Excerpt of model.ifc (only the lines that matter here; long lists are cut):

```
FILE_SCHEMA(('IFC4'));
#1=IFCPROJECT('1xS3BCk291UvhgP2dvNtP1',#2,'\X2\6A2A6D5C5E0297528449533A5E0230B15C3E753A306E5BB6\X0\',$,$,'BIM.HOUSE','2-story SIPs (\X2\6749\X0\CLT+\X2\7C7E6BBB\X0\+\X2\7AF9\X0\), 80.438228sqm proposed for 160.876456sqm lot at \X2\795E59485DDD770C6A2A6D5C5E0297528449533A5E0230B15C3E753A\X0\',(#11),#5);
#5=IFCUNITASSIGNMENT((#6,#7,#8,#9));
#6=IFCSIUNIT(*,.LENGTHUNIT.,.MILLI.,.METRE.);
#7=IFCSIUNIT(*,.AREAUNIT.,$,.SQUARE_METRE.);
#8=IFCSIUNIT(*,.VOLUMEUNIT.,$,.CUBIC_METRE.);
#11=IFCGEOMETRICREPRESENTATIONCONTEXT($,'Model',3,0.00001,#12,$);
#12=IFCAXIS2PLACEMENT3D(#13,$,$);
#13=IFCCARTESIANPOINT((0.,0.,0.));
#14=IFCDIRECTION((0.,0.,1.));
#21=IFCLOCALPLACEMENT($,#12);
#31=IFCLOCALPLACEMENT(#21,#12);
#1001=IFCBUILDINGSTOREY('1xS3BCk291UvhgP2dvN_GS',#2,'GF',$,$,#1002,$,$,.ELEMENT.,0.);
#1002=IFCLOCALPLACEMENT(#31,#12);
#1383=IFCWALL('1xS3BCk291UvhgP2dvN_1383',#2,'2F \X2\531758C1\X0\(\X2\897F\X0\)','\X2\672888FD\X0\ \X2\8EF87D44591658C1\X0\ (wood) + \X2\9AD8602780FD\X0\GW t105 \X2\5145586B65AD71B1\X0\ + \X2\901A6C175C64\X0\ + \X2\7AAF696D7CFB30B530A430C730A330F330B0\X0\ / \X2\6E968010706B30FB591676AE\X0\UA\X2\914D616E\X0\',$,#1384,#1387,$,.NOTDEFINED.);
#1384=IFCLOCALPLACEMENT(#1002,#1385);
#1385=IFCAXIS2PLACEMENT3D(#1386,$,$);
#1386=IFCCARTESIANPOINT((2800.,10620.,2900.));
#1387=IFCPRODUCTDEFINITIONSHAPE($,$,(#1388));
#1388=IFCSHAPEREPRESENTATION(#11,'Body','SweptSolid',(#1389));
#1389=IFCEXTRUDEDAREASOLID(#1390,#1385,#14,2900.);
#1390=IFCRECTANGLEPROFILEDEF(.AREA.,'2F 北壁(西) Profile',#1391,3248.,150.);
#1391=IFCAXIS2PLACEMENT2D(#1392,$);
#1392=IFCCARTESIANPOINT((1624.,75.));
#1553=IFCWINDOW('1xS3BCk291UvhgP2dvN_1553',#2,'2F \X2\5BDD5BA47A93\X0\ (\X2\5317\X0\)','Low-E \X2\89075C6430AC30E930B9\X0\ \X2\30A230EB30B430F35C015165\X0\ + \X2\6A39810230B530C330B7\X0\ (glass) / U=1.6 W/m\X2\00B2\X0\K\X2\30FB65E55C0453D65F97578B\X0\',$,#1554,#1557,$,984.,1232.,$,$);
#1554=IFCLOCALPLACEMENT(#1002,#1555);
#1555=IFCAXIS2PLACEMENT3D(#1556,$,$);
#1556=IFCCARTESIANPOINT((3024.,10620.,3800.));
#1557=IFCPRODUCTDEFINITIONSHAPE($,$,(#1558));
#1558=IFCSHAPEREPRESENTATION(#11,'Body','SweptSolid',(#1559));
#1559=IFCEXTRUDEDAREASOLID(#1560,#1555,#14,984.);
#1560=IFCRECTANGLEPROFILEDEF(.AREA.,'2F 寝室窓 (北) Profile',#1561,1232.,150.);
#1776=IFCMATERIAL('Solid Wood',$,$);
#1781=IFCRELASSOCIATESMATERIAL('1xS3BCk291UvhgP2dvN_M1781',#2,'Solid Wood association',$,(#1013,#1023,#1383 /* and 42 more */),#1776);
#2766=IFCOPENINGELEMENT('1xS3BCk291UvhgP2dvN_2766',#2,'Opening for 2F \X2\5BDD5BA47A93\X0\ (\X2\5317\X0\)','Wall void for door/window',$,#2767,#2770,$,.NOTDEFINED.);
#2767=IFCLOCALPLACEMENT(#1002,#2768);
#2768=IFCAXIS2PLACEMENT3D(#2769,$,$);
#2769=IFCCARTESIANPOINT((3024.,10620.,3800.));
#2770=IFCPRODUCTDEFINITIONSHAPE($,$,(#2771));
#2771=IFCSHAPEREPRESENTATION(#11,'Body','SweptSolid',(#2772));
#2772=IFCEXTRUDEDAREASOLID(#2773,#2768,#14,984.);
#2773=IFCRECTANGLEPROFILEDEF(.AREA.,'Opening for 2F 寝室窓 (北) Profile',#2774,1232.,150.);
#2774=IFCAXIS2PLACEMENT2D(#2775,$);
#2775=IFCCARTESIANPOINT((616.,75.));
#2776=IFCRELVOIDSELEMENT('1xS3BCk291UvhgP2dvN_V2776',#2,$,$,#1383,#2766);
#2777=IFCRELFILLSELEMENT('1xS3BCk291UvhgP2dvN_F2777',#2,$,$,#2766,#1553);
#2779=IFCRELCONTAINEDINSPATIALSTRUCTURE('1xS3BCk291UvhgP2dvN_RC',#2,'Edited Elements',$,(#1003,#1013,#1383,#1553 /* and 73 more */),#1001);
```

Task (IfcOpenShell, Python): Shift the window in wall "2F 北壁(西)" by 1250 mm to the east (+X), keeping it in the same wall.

```python
import ifcopenshell
import ifcopenshell.api.geometry
import ifcopenshell.util.placement

model = ifcopenshell.open("model.ifc")

window = model.by_guid("1xS3BCk291UvhgP2dvN_1553")
opening = window.FillsVoids[0].RelatingOpeningElement
wall = opening.VoidsElements[0].RelatingBuildingElement

wall_matrix = ifcopenshell.util.placement.get_local_placement(wall.ObjectPlacement)
shift = wall_matrix[:3, 0] * 1250.0
before = ifcopenshell.util.placement.get_local_placement(window.ObjectPlacement)[:3, 3].copy()

# The window is not placed relative to its opening, so move both.
for product in (opening, window):
    matrix = ifcopenshell.util.placement.get_local_placement(product.ObjectPlacement)
    matrix[:3, 3] += shift
    ifcopenshell.api.geometry.edit_object_placement(model, product=product, matrix=matrix, is_si=False)

after = ifcopenshell.util.placement.get_local_placement(window.ObjectPlacement)[:3, 3]
print("window moved by", (after - before).round(3) + 0.0)

model.write("model-out.ifc")
```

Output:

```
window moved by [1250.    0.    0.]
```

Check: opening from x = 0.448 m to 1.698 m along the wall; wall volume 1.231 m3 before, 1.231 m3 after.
